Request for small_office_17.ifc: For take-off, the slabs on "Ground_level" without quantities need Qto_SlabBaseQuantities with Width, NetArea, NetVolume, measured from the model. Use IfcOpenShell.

First a look at what the model holds.

```python
import ifcopenshell
import ifcopenshell.util.element
import ifcopenshell.util.unit

model = ifcopenshell.open("small_office_17.ifc")
print(model.schema)
for unit_type in ("LENGTHUNIT", "AREAUNIT", "VOLUMEUNIT"):
    print(unit_type, ifcopenshell.util.unit.calculate_unit_scale(model, unit_type))
storey = next(s for s in model.by_type("IfcBuildingStorey") if s.Name == "Ground_level")
slabs = [e for e in ifcopenshell.util.element.get_decomposition(storey) if e.is_a("IfcSlab")]
for e in sorted(slabs, key=lambda e: e.id()):
    print(e.id(), e.is_a(), e.Name, list(ifcopenshell.util.element.get_psets(e, qtos_only=True)), sep=" | ")
```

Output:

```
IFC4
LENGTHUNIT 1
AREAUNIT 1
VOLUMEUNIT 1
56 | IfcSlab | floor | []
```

```python
import ifcopenshell
import ifcopenshell.api.pset
import ifcopenshell.geom
import ifcopenshell.util.element
import ifcopenshell.util.shape
import ifcopenshell.util.unit

model = ifcopenshell.open("small_office_17.ifc")
unit_scale = ifcopenshell.util.unit.calculate_unit_scale(model)
area_scale = ifcopenshell.util.unit.calculate_unit_scale(model, "AREAUNIT")
volume_scale = ifcopenshell.util.unit.calculate_unit_scale(model, "VOLUMEUNIT")
settings = ifcopenshell.geom.settings()

storey = next(s for s in model.by_type("IfcBuildingStorey") if s.Name == "Ground_level")
slabs = [e for e in ifcopenshell.util.element.get_decomposition(storey) if e.is_a("IfcSlab")]

for e in sorted(slabs, key=lambda e: e.id()):
    if ifcopenshell.util.element.get_psets(e, qtos_only=True, should_inherit=False):
        continue
    # Geometry comes back in metres, in the element's own axes.
    shape = ifcopenshell.geom.create_shape(settings, e)
    values = {
        "Width": ifcopenshell.util.shape.get_z(shape.geometry) / unit_scale,
        "NetArea": ifcopenshell.util.shape.get_footprint_area(shape.geometry) / area_scale,
        "NetVolume": ifcopenshell.util.shape.get_volume(shape.geometry) / volume_scale,
    }
    qto = ifcopenshell.api.pset.add_qto(model, product=e, name="Qto_SlabBaseQuantities")
    ifcopenshell.api.pset.edit_qto(model, qto=qto, properties=values)
    print(e.id(), {k: round(v, 3) for k, v in values.items()})

model.write("small_office_17_rev.ifc")
```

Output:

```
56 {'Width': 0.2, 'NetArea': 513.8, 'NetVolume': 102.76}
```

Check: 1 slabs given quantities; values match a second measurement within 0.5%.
